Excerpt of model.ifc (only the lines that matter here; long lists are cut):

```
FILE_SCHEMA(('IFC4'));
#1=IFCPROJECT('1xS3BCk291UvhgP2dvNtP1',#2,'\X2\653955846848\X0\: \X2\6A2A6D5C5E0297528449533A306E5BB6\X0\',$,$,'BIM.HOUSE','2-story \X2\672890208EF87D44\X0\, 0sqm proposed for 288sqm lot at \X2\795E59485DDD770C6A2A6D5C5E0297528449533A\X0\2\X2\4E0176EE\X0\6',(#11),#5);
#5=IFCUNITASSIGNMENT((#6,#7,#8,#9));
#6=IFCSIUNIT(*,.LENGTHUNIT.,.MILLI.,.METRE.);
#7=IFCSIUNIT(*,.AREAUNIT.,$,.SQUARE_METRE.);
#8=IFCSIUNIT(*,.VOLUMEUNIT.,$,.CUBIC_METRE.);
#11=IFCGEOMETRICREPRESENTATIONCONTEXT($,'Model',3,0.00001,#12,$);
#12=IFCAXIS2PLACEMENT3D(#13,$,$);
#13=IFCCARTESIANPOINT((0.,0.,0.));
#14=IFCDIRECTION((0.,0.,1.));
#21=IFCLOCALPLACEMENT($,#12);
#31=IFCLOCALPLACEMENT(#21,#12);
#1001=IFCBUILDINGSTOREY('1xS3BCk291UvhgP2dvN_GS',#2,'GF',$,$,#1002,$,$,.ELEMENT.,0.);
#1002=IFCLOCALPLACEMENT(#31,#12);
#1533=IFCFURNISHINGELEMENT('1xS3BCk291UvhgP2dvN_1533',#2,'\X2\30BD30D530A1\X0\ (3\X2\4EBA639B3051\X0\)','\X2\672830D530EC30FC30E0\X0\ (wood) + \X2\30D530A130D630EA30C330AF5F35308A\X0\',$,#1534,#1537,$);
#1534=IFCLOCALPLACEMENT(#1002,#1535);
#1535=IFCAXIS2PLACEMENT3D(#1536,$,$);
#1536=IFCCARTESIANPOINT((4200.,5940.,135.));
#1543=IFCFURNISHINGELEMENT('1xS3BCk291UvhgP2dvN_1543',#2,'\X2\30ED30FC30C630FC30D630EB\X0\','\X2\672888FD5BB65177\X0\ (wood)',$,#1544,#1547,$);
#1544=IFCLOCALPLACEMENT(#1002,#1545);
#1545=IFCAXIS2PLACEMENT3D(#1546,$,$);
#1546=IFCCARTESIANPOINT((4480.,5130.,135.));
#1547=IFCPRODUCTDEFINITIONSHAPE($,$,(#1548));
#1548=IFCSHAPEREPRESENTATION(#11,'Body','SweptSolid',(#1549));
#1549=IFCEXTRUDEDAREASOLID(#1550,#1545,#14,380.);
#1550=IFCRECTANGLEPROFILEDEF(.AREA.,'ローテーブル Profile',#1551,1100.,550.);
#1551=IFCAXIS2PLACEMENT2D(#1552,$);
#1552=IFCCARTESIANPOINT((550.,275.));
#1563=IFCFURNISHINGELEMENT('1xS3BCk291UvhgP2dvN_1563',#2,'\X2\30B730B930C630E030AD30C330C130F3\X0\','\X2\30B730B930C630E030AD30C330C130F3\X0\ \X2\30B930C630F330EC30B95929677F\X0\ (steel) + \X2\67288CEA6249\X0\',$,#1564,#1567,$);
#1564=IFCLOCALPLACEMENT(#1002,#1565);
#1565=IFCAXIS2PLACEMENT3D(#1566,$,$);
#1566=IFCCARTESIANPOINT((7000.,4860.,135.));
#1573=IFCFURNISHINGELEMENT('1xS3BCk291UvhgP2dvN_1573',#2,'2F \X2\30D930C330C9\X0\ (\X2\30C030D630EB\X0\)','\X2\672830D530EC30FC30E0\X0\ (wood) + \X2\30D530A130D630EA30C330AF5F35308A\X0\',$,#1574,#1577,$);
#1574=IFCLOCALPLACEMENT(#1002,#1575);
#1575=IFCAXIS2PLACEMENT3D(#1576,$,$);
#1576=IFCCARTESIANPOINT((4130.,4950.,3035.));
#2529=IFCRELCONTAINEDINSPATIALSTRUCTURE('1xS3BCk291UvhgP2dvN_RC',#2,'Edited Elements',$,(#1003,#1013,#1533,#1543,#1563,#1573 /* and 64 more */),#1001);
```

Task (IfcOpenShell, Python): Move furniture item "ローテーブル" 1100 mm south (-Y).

```python
import ifcopenshell
import ifcopenshell.api.geometry
import ifcopenshell.util.placement

model = ifcopenshell.open("model.ifc")

item = model.by_id(1543)
matrix = ifcopenshell.util.placement.get_local_placement(item.ObjectPlacement)
matrix[1, 3] -= 1100.0
ifcopenshell.api.geometry.edit_object_placement(model, product=item, matrix=matrix, is_si=False)

print(ifcopenshell.util.placement.get_local_placement(item.ObjectPlacement).round(3) + 0.0)

model.write("model_v2.ifc")
```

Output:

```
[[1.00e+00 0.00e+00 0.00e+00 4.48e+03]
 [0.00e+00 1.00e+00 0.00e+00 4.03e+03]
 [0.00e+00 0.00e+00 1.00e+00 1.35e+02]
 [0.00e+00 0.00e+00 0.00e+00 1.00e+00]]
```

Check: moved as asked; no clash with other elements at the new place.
